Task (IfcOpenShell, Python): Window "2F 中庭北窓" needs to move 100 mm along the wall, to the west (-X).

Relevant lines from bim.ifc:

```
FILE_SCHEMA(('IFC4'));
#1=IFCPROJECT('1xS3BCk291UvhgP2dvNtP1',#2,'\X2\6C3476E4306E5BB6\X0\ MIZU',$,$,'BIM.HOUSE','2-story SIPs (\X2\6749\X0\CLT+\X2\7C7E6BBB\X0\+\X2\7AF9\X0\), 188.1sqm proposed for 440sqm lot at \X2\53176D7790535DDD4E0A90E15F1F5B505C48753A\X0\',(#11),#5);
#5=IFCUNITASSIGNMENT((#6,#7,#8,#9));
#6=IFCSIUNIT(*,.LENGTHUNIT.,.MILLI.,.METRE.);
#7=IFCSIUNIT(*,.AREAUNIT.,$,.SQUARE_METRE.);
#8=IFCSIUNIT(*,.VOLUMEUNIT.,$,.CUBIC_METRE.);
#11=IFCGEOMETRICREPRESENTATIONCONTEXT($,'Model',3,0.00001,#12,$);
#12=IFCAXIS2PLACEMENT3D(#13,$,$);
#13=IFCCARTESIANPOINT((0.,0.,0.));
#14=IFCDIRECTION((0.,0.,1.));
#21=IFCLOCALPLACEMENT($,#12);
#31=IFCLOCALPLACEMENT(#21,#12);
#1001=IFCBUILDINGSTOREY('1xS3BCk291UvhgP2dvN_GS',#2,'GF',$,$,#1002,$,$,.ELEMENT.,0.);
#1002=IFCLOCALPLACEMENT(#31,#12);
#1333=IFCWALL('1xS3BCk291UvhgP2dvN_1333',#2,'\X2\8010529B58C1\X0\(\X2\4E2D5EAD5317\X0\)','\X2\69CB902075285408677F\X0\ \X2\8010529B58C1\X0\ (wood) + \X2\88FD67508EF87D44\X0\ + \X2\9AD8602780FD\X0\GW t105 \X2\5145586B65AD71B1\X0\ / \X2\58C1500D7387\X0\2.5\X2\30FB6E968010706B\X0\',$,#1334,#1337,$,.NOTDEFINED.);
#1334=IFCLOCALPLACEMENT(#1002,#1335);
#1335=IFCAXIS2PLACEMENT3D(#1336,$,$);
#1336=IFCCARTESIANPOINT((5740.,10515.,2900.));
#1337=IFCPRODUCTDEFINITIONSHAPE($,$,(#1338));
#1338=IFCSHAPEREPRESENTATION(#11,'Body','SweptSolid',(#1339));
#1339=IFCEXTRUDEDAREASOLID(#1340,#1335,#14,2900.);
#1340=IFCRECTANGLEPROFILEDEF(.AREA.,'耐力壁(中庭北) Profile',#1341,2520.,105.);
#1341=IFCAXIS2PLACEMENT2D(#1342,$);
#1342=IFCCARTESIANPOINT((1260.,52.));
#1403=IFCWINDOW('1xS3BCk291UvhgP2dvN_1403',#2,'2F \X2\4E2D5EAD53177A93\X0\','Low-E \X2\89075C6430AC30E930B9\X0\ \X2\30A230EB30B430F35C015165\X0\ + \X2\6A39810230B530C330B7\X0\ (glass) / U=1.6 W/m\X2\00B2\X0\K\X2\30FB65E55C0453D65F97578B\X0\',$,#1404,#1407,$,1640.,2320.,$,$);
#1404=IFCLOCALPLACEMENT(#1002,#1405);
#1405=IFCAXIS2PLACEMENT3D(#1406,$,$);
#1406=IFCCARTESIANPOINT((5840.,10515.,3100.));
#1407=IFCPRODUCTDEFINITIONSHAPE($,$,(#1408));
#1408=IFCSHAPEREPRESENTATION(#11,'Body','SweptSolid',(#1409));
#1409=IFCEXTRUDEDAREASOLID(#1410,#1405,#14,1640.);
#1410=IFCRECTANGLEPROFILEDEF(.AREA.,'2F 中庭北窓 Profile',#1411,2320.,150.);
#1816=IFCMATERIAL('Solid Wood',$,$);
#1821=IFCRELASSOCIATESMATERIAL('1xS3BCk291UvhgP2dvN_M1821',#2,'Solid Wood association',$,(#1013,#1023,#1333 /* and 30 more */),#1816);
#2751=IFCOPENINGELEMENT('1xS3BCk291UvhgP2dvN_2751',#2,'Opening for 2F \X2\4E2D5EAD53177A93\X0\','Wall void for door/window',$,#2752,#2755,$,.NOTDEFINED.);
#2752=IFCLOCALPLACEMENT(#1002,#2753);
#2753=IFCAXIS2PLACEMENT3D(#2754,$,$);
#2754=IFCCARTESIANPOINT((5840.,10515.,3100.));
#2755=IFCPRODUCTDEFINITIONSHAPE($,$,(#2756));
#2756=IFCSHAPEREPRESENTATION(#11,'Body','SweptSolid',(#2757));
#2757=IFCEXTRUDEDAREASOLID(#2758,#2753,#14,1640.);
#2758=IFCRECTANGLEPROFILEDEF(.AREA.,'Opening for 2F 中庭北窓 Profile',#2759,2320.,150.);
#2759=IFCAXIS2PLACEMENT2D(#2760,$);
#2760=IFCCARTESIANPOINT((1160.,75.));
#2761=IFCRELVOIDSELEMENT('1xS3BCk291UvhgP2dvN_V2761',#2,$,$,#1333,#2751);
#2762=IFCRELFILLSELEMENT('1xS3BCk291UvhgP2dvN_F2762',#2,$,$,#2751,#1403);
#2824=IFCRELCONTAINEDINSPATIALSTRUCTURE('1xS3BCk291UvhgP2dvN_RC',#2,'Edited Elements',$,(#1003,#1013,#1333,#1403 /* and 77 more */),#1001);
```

```python
import ifcopenshell
import ifcopenshell.api.geometry
import ifcopenshell.util.placement

model = ifcopenshell.open("bim.ifc")

window = model.by_guid("1xS3BCk291UvhgP2dvN_1403")
opening = window.FillsVoids[0].RelatingOpeningElement
wall = opening.VoidsElements[0].RelatingBuildingElement

wall_matrix = ifcopenshell.util.placement.get_local_placement(wall.ObjectPlacement)
shift = wall_matrix[:3, 0] * -100.0
before = ifcopenshell.util.placement.get_local_placement(window.ObjectPlacement)[:3, 3].copy()

# The window is not placed relative to its opening, so move both.
for product in (opening, window):
    matrix = ifcopenshell.util.placement.get_local_placement(product.ObjectPlacement)
    matrix[:3, 3] += shift
    ifcopenshell.api.geometry.edit_object_placement(model, product=product, matrix=matrix, is_si=False)

after = ifcopenshell.util.placement.get_local_placement(window.ObjectPlacement)[:3, 3]
print("window moved by", (after - before).round(3) + 0.0)

model.write("bim_edited.ifc")
```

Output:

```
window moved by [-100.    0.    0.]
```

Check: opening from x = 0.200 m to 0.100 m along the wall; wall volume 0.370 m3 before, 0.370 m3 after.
